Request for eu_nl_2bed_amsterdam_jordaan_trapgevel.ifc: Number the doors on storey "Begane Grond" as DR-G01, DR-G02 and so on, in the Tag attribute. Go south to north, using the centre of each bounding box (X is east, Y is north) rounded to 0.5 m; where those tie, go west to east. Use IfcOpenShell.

First a look at what the model holds.

```python
import ifcopenshell
import ifcopenshell.util.element
import ifcopenshell.util.placement

model = ifcopenshell.open("eu_nl_2bed_amsterdam_jordaan_trapgevel.ifc")
print(model.schema)
storey = next(s for s in model.by_type("IfcBuildingStorey") if s.Name == "Begane Grond")
doors = [e for e in ifcopenshell.util.element.get_decomposition(storey) if e.is_a("IfcDoor")]
for e in sorted(doors, key=lambda e: e.id()):
    origin = ifcopenshell.util.placement.get_local_placement(e.ObjectPlacement)[:3, 3]
    print(e.id(), e.Tag, e.Name, origin.round(2) + 0.0, sep=" | ")
```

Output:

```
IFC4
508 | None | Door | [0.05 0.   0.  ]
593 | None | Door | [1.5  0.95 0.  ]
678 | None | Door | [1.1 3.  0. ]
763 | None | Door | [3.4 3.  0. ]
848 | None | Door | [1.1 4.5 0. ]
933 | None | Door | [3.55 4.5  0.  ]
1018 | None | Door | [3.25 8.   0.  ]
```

```python
import ifcopenshell
import ifcopenshell.geom
import ifcopenshell.util.element
import ifcopenshell.util.shape

model = ifcopenshell.open("eu_nl_2bed_amsterdam_jordaan_trapgevel.ifc")
settings = ifcopenshell.geom.settings()
settings.set("use-world-coords", True)


def centre(element):
    shape = ifcopenshell.geom.create_shape(settings, element)
    return ifcopenshell.util.shape.get_bbox_centroid(shape.geometry)


storey = next(s for s in model.by_type("IfcBuildingStorey") if s.Name == "Begane Grond")
doors = [e for e in ifcopenshell.util.element.get_decomposition(storey) if e.is_a("IfcDoor")]

# Insertion points can sit at a corner or the storey origin, so sort by the geometry (in metres).
centres = {e: centre(e) for e in doors}
doors.sort(key=lambda e: (round(centres[e][1] / 0.5), centres[e][0]))

for i, e in enumerate(doors, start=1):
    number = f"DR-G{i:02d}"
    e.Tag = number
    print(e.id(), number)

model.write("eu_nl_2bed_amsterdam_jordaan_trapgevel_updated.ifc")
```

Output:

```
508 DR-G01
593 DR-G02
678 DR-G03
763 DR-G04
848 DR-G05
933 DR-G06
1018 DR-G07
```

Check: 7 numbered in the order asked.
